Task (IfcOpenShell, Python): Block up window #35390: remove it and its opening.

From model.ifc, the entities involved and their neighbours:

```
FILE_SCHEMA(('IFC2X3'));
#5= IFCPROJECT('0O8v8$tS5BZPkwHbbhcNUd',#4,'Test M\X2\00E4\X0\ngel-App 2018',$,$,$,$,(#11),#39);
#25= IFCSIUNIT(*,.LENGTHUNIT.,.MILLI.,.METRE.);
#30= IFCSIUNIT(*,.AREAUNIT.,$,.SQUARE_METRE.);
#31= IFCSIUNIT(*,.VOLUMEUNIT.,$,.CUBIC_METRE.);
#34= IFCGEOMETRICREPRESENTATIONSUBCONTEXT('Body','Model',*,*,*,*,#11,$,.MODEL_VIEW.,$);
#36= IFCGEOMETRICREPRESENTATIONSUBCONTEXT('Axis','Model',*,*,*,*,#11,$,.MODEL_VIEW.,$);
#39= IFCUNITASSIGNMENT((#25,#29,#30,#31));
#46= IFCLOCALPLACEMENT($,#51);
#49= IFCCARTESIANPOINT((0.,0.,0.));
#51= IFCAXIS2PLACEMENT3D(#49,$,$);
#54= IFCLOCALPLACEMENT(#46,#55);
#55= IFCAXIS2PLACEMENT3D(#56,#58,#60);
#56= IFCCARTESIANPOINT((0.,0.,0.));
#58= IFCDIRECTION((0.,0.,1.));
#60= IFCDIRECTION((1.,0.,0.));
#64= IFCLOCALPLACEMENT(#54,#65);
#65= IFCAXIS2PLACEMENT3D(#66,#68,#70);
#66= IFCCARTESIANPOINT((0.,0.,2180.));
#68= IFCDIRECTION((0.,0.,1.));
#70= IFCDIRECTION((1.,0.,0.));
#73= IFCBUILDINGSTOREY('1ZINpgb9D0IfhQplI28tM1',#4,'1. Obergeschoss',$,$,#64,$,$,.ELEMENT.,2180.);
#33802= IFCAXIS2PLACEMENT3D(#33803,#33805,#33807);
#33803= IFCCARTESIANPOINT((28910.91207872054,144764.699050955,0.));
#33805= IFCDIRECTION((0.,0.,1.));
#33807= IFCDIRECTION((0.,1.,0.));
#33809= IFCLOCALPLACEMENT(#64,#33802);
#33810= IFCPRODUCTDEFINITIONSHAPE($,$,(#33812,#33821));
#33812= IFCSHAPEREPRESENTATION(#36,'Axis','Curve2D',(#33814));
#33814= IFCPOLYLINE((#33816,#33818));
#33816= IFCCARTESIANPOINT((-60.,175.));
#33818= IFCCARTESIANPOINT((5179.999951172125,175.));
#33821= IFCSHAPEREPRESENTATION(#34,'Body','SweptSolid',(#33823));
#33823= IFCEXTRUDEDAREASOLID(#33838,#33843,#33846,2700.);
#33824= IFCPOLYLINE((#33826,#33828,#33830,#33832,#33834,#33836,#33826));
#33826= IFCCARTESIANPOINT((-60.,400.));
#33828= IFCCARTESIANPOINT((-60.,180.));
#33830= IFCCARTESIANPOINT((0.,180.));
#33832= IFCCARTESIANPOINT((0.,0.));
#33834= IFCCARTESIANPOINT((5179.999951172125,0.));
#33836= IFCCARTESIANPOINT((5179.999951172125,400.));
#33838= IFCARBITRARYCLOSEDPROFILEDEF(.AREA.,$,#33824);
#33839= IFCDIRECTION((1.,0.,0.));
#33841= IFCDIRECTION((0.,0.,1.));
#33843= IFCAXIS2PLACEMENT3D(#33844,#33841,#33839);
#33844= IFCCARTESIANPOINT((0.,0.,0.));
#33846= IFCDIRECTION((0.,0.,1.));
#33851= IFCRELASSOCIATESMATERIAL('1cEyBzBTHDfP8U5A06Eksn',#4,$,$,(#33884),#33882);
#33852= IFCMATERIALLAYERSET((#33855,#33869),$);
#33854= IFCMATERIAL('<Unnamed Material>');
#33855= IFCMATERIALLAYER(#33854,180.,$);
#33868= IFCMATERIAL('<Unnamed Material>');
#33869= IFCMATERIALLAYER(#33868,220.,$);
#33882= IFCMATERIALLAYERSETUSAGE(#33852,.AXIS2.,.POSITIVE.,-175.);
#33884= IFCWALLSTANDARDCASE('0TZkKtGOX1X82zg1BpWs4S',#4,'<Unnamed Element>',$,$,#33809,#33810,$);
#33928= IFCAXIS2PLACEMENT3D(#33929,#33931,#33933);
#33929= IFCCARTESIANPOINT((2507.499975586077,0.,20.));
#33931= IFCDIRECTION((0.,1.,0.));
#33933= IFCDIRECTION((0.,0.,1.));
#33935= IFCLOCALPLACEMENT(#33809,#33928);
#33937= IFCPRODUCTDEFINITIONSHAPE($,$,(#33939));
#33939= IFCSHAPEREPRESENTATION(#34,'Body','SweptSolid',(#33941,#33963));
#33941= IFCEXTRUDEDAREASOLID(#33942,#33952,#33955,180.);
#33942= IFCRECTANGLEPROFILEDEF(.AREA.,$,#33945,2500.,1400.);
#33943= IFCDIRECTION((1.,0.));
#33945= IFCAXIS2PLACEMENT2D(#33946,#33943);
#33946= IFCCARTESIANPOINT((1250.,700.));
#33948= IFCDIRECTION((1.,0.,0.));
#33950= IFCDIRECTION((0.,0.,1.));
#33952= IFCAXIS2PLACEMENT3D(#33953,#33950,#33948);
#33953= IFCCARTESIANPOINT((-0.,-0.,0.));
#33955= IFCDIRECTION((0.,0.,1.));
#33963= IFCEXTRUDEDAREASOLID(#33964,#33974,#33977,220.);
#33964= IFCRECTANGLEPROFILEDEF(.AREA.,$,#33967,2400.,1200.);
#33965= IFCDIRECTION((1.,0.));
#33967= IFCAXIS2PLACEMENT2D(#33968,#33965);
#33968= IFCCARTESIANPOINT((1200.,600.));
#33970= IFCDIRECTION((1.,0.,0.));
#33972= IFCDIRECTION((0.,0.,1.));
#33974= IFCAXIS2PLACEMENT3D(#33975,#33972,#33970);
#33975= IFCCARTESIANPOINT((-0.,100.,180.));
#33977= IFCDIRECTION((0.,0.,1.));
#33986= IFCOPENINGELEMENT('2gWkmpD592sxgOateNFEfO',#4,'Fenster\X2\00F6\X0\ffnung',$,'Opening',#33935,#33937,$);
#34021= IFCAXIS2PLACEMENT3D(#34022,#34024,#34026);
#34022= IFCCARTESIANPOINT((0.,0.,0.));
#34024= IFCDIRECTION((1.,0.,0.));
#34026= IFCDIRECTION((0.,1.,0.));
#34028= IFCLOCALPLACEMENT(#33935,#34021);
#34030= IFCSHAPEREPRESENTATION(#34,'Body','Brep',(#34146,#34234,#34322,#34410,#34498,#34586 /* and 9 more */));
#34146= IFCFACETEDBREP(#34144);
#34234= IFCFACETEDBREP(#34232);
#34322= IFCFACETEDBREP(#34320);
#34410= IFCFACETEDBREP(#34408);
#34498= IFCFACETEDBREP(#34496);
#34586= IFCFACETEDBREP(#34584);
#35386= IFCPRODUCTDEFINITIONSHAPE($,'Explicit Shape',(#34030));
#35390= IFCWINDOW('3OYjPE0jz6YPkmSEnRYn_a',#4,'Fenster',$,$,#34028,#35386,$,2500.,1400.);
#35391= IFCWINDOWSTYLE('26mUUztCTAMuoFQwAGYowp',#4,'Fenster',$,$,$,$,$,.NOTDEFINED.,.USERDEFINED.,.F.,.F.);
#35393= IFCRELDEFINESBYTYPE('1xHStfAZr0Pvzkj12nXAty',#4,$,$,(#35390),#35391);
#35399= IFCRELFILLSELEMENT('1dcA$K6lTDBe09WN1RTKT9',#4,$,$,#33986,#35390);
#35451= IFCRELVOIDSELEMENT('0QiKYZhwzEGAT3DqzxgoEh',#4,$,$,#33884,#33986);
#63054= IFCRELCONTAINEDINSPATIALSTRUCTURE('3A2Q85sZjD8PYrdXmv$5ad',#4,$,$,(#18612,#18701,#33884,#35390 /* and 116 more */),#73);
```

```python
import ifcopenshell
import ifcopenshell.api.feature
import ifcopenshell.api.root
import ifcopenshell.geom
import ifcopenshell.util.shape

model = ifcopenshell.open("model.ifc")
settings = ifcopenshell.geom.settings()


def volume(element):
    """Net volume in cubic metres, openings subtracted."""
    shape = ifcopenshell.geom.create_shape(settings, element)
    return ifcopenshell.util.shape.get_volume(shape.geometry)


window = model.by_id(35390)
opening = window.FillsVoids[0].RelatingOpeningElement
wall = opening.VoidsElements[0].RelatingBuildingElement
before = volume(wall)

ifcopenshell.api.root.remove_product(model, product=window)
ifcopenshell.api.feature.remove_feature(model, feature=opening)

after = volume(wall)

print(f"wall volume {before:.3f} -> {after:.3f} m3")

model.write("model_updated.ifc")
```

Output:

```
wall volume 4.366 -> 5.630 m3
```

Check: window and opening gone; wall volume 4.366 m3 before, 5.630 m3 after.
